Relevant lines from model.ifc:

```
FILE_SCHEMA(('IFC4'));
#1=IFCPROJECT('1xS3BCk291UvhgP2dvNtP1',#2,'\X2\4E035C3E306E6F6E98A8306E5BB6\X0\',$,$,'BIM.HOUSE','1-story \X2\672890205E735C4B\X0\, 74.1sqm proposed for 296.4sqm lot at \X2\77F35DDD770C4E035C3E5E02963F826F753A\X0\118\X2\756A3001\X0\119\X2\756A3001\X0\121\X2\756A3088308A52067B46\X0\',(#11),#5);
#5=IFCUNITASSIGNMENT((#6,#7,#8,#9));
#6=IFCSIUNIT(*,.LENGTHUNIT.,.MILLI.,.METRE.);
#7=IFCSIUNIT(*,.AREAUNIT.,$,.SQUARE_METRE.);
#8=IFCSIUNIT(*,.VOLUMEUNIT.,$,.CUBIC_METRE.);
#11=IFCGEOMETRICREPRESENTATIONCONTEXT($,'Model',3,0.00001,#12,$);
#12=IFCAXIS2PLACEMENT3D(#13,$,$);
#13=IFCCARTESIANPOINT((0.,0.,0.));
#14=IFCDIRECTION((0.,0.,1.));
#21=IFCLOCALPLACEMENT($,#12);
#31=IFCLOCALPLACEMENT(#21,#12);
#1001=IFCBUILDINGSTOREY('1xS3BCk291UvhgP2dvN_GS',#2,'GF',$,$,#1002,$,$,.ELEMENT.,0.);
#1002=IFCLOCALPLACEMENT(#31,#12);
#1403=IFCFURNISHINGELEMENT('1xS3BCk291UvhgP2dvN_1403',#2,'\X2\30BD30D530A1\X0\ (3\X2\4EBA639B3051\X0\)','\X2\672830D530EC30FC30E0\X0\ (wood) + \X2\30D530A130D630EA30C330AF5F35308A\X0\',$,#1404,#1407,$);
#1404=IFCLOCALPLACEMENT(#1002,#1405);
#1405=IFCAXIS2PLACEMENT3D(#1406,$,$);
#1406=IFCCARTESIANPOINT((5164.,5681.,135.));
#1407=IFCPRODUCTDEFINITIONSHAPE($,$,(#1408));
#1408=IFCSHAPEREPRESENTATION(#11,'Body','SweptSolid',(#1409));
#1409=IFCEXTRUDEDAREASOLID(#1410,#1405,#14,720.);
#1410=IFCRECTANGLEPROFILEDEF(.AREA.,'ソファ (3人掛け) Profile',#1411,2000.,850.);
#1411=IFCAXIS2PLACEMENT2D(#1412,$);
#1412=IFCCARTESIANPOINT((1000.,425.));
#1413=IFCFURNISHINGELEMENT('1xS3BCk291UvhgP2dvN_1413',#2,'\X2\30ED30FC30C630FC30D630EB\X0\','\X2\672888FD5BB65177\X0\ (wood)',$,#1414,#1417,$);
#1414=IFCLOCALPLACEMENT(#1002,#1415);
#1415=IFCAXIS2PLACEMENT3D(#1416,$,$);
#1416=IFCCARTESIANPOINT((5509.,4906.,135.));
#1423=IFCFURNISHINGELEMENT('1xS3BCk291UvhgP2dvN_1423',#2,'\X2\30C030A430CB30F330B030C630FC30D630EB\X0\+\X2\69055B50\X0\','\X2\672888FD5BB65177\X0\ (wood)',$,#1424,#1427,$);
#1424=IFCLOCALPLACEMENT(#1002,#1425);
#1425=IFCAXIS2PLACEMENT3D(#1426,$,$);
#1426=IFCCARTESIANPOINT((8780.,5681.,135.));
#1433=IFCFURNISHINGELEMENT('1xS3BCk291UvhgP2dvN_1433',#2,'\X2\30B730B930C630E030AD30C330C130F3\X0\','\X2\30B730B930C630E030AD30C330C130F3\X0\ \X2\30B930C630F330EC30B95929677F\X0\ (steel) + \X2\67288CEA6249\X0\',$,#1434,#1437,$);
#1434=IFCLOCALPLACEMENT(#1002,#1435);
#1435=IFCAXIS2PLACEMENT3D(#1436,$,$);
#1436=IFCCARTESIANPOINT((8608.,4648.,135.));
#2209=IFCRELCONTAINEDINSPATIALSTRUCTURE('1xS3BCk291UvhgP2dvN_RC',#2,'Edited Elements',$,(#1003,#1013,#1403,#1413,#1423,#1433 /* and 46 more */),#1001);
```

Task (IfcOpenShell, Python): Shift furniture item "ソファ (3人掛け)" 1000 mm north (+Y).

```python
import ifcopenshell
import ifcopenshell.api.geometry
import ifcopenshell.util.placement
import ifcopenshell.util.unit

model = ifcopenshell.open("model.ifc")
unit_scale = ifcopenshell.util.unit.calculate_unit_scale(model)

item = model.by_guid("1xS3BCk291UvhgP2dvN_1403")
matrix = ifcopenshell.util.placement.get_local_placement(item.ObjectPlacement)
matrix[1, 3] += 1 / unit_scale
ifcopenshell.api.geometry.edit_object_placement(model, product=item, matrix=matrix, is_si=False)

print(ifcopenshell.util.placement.get_local_placement(item.ObjectPlacement).round(3) + 0.0)

model.write("model-out.ifc")
```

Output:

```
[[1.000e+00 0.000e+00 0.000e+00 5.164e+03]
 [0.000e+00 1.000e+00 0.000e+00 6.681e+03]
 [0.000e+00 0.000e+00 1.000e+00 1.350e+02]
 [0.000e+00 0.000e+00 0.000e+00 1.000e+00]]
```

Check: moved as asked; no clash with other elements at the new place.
